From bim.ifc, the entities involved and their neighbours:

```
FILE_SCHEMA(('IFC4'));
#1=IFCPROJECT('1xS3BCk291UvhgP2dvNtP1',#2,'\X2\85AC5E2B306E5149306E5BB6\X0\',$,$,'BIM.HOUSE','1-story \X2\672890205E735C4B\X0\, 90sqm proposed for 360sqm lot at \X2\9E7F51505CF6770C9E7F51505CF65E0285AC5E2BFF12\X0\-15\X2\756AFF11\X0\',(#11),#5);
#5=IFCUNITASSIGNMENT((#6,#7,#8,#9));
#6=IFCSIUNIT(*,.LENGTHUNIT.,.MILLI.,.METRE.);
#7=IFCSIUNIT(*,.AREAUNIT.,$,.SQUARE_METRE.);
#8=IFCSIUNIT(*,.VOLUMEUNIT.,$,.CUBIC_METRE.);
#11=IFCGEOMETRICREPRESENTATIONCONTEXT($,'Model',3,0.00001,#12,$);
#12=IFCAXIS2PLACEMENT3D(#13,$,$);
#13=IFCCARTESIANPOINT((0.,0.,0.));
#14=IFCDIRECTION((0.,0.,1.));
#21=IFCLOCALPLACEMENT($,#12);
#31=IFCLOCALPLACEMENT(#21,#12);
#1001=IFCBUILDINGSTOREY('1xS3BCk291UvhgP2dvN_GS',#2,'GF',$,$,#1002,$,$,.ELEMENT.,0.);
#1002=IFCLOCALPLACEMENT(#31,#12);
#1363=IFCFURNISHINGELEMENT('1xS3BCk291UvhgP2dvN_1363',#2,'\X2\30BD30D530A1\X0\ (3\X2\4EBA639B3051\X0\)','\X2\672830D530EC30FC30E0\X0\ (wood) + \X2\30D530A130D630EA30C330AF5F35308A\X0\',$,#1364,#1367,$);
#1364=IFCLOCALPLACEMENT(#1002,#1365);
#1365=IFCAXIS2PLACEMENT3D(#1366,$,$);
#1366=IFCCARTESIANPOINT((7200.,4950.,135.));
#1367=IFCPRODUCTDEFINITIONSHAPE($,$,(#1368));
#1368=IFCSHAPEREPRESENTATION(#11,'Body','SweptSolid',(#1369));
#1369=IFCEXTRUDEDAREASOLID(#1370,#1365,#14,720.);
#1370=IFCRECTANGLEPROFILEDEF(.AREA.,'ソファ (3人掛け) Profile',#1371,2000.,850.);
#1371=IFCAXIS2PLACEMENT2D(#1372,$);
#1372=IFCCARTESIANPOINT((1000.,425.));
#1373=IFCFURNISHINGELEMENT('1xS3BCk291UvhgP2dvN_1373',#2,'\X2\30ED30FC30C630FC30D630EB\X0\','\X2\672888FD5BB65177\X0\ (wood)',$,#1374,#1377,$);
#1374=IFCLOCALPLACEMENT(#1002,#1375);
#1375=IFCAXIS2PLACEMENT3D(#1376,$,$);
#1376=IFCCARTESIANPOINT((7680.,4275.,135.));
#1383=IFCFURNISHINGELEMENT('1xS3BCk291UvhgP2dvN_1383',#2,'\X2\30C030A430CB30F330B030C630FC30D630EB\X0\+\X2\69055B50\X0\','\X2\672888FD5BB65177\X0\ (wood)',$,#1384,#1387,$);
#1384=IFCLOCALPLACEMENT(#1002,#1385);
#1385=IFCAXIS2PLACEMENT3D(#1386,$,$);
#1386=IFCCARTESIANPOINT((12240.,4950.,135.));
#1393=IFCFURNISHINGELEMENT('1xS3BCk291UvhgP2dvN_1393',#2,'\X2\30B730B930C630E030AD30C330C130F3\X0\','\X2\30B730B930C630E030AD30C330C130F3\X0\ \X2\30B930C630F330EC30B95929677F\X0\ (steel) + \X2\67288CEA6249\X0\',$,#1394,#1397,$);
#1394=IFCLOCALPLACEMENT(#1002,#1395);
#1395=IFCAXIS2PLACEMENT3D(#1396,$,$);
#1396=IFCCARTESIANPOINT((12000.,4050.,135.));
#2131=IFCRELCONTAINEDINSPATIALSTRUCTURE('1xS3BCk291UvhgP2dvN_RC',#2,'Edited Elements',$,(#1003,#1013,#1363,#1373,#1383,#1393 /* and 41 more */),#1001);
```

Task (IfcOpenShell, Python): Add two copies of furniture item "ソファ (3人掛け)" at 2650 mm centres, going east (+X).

```python
import numpy as np
import ifcopenshell
import ifcopenshell.api.geometry
import ifcopenshell.api.root
import ifcopenshell.util.element
import ifcopenshell.util.placement
import ifcopenshell.util.unit

model = ifcopenshell.open("bim.ifc")
unit_scale = ifcopenshell.util.unit.calculate_unit_scale(model)


def reuse_history(source, copy):
    """copy_class also copies each property set's owner history, people and application; keep the originals."""
    for rel in copy.IsDefinedBy:
        if rel.is_a("IfcRelDefinesByProperties") and (history := rel.RelatingPropertyDefinition.OwnerHistory):
            rel.RelatingPropertyDefinition.OwnerHistory = source.OwnerHistory
            ifcopenshell.util.element.remove_deep2(model, history)


source = model.by_id(1363)
base = ifcopenshell.util.placement.get_local_placement(source.ObjectPlacement)
step = np.array([1.0, 0.0, 0.0]) * 2.65 / unit_scale

for i in range(1, 3):
    copy = ifcopenshell.api.root.copy_class(model, product=source)
    copy.Representation = ifcopenshell.util.element.copy_deep(
        model, source.Representation, exclude=["IfcGeometricRepresentationContext", "IfcRepresentationMap"]
    )
    reuse_history(source, copy)
    matrix = base.copy()
    matrix[:3, 3] += i * step
    print("added at", matrix[:3, 3].round(3) + 0.0)
    ifcopenshell.api.geometry.edit_object_placement(model, product=copy, matrix=matrix, is_si=False)

model.write("bim_updated.ifc")
```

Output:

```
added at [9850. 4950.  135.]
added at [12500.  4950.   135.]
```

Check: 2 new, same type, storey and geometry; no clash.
